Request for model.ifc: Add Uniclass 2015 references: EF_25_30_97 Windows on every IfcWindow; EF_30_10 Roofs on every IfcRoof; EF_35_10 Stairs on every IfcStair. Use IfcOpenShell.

First a look at what the model holds.

```python
import ifcopenshell

model = ifcopenshell.open("model.ifc")
print(model.schema)
print("classifications:", [c.Name for c in model.by_type("IfcClassification")])
for ifc_class in ("IfcDoor", "IfcRoof", "IfcStair", "IfcWall", "IfcWindow"):
    print(ifc_class, len(model.by_type(ifc_class)))
```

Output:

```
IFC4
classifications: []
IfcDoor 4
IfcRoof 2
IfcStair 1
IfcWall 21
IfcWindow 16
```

```python
import ifcopenshell
import ifcopenshell.api.classification

model = ifcopenshell.open("model.ifc")

system = ifcopenshell.api.classification.add_classification(model, classification="Uniclass 2015")

codes = {
    "IfcWindow": ("EF_25_30_97", "Windows"),
    "IfcRoof": ("EF_30_10", "Roofs"),
    "IfcStair": ("EF_35_10", "Stairs"),
}
for ifc_class, (code, name) in codes.items():
    products = model.by_type(ifc_class)
    ifcopenshell.api.classification.add_reference(
        model, products=products, classification=system, identification=code, name=name
    )
    print(code, len(products))

model.write("model_edited.ifc")
```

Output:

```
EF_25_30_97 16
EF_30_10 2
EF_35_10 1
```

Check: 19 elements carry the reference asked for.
